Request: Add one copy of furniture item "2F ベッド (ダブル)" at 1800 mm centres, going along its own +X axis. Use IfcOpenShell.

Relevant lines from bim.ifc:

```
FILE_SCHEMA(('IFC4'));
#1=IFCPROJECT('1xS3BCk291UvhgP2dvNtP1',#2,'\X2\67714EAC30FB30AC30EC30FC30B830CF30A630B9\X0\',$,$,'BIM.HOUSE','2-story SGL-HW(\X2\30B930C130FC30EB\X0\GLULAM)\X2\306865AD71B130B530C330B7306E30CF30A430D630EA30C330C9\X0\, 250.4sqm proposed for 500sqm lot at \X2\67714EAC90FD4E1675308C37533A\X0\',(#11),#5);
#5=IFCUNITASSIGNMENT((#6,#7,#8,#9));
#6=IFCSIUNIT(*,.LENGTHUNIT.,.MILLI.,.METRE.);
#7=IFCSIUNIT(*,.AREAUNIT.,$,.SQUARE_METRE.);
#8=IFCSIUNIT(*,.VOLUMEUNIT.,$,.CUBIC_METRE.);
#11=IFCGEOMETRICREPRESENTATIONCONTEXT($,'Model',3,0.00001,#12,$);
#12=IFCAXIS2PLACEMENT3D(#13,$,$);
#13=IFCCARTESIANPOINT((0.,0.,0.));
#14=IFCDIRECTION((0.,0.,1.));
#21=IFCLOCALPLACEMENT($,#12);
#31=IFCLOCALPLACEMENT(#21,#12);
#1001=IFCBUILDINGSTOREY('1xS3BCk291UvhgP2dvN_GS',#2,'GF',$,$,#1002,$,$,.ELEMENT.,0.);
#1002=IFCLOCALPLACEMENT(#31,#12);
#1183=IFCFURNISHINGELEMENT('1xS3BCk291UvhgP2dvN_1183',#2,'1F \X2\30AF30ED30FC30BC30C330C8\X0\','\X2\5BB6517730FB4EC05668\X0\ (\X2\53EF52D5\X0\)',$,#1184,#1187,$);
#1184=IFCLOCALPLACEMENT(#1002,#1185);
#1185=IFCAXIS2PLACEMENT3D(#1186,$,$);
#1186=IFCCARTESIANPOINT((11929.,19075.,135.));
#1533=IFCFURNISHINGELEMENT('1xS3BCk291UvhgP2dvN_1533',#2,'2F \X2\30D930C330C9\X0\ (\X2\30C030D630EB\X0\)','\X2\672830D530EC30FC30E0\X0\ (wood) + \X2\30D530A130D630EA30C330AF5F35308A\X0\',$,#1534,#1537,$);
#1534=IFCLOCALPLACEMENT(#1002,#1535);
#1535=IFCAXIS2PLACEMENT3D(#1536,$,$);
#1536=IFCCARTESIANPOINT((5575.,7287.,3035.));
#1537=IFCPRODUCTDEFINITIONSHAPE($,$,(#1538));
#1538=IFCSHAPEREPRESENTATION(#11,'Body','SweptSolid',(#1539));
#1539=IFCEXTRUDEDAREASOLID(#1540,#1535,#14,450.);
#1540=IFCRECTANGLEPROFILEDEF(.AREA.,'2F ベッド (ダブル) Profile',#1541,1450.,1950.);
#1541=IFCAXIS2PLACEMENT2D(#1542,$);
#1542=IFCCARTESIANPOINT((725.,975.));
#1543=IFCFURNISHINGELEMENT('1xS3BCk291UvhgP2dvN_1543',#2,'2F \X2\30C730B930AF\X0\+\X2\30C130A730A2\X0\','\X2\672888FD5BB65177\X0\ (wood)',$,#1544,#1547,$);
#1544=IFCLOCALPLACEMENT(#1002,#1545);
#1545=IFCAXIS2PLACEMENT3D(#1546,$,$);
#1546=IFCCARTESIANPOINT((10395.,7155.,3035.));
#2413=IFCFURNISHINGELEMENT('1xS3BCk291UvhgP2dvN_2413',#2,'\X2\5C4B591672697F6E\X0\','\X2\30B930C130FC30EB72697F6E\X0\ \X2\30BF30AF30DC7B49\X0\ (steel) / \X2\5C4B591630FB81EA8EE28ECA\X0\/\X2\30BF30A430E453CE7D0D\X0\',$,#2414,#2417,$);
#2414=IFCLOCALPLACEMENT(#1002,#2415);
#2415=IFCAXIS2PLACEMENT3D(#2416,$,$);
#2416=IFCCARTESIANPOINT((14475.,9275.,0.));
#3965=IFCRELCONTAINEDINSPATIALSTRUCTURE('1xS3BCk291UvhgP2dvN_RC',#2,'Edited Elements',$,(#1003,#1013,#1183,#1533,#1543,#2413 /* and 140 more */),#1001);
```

```python
import ifcopenshell
import ifcopenshell.api.geometry
import ifcopenshell.api.root
import ifcopenshell.util.element
import ifcopenshell.util.placement
import ifcopenshell.util.unit

model = ifcopenshell.open("bim.ifc")
unit_scale = ifcopenshell.util.unit.calculate_unit_scale(model)


def reuse_history(source, copy):
    """copy_class also copies each property set's owner history, people and application; keep the originals."""
    for rel in copy.IsDefinedBy:
        if rel.is_a("IfcRelDefinesByProperties") and (history := rel.RelatingPropertyDefinition.OwnerHistory):
            rel.RelatingPropertyDefinition.OwnerHistory = source.OwnerHistory
            ifcopenshell.util.element.remove_deep2(model, history)


source = model.by_guid("1xS3BCk291UvhgP2dvN_1533")
base = ifcopenshell.util.placement.get_local_placement(source.ObjectPlacement)
step = base[:3, 0] * 1.8 / unit_scale

for i in range(1, 2):
    copy = ifcopenshell.api.root.copy_class(model, product=source)
    copy.Representation = ifcopenshell.util.element.copy_deep(
        model, source.Representation, exclude=["IfcGeometricRepresentationContext", "IfcRepresentationMap"]
    )
    reuse_history(source, copy)
    matrix = base.copy()
    matrix[:3, 3] += i * step
    print("added at", matrix[:3, 3].round(3) + 0.0)
    ifcopenshell.api.geometry.edit_object_placement(model, product=copy, matrix=matrix, is_si=False)

model.write("bim_updated.ifc")
```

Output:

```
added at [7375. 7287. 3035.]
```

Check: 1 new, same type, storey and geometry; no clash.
